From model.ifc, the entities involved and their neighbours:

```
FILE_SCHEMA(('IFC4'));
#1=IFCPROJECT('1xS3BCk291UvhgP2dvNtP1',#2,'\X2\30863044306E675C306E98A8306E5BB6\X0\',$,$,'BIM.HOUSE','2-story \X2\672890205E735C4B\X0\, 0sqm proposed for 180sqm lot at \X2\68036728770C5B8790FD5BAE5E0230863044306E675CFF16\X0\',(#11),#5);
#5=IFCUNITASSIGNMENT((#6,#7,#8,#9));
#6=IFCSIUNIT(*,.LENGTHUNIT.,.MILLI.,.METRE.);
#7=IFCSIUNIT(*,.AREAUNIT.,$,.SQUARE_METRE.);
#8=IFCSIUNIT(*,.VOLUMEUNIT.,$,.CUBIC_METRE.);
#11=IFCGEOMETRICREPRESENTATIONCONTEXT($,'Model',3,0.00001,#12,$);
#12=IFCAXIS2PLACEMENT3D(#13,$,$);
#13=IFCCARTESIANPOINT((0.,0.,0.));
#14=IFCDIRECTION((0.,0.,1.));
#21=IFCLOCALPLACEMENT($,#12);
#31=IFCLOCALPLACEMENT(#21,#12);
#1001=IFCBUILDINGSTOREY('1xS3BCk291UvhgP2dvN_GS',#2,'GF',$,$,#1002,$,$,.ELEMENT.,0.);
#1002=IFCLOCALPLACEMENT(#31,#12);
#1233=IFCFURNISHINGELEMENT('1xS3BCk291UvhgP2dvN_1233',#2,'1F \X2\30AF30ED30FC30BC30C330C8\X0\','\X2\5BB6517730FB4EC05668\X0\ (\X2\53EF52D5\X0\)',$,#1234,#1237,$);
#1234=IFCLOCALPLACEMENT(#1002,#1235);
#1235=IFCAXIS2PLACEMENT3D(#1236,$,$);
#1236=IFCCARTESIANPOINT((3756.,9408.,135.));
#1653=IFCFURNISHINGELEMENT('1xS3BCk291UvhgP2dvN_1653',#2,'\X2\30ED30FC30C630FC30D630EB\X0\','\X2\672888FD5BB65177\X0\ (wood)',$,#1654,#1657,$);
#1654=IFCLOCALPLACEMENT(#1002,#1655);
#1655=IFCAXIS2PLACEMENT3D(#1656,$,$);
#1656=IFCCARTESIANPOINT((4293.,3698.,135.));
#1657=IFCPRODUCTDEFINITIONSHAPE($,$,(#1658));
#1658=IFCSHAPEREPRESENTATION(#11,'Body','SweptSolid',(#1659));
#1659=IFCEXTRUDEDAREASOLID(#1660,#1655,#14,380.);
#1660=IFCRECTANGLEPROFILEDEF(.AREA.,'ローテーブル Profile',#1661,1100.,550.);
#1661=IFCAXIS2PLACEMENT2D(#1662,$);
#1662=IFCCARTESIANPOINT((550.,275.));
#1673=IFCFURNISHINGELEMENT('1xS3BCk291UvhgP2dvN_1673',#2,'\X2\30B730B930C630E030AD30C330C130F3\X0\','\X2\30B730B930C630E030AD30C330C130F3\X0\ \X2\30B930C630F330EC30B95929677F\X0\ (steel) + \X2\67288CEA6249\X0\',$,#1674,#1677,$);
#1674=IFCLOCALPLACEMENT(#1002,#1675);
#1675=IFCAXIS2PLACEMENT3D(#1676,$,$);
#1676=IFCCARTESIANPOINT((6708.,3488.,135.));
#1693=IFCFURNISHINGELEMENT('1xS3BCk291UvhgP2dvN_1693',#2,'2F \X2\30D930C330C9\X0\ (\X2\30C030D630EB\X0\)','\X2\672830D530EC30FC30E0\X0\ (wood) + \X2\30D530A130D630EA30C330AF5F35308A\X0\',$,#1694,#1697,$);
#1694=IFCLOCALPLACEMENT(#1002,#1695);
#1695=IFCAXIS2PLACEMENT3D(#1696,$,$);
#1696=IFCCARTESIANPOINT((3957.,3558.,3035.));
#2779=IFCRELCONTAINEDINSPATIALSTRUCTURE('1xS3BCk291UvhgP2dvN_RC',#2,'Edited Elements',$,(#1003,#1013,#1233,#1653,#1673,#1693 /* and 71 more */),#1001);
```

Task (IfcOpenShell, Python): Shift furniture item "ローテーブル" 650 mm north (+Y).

```python
import ifcopenshell
import ifcopenshell.api.geometry
import ifcopenshell.util.placement
import ifcopenshell.util.unit

model = ifcopenshell.open("model.ifc")
unit_scale = ifcopenshell.util.unit.calculate_unit_scale(model)

item = model.by_guid("1xS3BCk291UvhgP2dvN_1653")
matrix = ifcopenshell.util.placement.get_local_placement(item.ObjectPlacement)
matrix[1, 3] += 0.65 / unit_scale
ifcopenshell.api.geometry.edit_object_placement(model, product=item, matrix=matrix, is_si=False)

print(ifcopenshell.util.placement.get_local_placement(item.ObjectPlacement).round(3) + 0.0)

model.write("model_v2.ifc")
```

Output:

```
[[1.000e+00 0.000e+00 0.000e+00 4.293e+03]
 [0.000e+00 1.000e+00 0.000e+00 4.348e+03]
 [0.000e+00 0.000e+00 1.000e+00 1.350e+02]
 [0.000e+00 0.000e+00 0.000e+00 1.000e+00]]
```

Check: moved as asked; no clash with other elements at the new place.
